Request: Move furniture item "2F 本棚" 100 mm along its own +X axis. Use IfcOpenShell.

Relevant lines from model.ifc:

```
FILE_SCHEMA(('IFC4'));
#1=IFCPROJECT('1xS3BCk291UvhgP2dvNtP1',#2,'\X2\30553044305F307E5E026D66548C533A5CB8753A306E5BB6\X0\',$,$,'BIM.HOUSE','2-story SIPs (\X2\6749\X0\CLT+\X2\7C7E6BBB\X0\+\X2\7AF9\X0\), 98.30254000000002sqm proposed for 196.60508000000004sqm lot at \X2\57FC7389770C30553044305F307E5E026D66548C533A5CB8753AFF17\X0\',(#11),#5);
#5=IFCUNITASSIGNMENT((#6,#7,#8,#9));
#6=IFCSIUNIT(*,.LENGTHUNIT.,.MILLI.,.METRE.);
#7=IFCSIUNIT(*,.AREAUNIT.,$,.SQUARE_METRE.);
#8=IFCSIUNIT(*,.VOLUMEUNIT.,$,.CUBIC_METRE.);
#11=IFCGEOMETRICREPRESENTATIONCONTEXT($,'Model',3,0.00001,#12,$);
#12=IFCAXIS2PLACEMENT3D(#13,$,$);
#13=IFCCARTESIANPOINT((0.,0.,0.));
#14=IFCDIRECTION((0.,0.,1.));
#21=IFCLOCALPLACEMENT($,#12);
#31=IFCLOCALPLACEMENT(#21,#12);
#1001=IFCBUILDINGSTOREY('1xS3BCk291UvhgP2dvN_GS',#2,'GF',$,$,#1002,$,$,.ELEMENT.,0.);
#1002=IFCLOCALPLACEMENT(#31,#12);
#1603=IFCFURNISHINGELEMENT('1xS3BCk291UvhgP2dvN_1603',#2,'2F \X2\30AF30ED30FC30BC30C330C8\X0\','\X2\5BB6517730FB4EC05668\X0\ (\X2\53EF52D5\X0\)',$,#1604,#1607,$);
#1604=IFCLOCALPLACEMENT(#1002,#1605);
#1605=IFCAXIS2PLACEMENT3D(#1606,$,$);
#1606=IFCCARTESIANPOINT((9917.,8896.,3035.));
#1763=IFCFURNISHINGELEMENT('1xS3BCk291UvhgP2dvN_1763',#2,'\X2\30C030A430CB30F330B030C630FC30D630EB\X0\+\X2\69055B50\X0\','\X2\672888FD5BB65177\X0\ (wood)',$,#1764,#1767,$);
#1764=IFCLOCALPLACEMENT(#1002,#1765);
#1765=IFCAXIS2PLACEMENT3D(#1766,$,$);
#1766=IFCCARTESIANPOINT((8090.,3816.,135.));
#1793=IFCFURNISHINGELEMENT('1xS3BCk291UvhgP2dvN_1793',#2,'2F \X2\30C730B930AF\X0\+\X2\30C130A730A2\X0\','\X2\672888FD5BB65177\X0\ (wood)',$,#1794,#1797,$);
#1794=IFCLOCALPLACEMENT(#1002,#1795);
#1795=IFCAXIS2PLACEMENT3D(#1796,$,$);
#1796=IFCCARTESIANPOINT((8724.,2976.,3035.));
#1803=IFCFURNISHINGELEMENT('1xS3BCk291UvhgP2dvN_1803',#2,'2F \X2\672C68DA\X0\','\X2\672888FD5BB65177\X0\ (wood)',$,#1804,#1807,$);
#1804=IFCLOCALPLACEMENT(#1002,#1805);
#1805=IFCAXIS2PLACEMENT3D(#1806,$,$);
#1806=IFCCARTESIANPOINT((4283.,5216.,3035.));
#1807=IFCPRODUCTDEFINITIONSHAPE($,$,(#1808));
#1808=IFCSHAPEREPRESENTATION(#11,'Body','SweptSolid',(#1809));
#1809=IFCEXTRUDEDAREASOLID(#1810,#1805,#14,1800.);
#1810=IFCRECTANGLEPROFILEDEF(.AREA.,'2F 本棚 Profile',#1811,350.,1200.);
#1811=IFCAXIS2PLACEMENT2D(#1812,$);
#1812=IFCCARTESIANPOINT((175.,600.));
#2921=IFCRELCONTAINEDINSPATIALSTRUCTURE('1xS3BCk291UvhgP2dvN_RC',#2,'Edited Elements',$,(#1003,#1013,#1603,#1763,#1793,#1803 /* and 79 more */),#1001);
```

```python
import ifcopenshell
import ifcopenshell.api.geometry
import ifcopenshell.util.placement

model = ifcopenshell.open("model.ifc")

item = model.by_guid("1xS3BCk291UvhgP2dvN_1803")
matrix = ifcopenshell.util.placement.get_local_placement(item.ObjectPlacement)
matrix[:3, 3] += matrix[:3, 0] * 100.0
ifcopenshell.api.geometry.edit_object_placement(model, product=item, matrix=matrix, is_si=False)

print(ifcopenshell.util.placement.get_local_placement(item.ObjectPlacement).round(3) + 0.0)

model.write("model_edited.ifc")
```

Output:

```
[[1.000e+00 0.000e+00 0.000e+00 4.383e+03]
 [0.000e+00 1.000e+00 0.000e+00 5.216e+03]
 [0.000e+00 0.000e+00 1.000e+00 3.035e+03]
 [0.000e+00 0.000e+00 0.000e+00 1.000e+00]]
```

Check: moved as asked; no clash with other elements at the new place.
